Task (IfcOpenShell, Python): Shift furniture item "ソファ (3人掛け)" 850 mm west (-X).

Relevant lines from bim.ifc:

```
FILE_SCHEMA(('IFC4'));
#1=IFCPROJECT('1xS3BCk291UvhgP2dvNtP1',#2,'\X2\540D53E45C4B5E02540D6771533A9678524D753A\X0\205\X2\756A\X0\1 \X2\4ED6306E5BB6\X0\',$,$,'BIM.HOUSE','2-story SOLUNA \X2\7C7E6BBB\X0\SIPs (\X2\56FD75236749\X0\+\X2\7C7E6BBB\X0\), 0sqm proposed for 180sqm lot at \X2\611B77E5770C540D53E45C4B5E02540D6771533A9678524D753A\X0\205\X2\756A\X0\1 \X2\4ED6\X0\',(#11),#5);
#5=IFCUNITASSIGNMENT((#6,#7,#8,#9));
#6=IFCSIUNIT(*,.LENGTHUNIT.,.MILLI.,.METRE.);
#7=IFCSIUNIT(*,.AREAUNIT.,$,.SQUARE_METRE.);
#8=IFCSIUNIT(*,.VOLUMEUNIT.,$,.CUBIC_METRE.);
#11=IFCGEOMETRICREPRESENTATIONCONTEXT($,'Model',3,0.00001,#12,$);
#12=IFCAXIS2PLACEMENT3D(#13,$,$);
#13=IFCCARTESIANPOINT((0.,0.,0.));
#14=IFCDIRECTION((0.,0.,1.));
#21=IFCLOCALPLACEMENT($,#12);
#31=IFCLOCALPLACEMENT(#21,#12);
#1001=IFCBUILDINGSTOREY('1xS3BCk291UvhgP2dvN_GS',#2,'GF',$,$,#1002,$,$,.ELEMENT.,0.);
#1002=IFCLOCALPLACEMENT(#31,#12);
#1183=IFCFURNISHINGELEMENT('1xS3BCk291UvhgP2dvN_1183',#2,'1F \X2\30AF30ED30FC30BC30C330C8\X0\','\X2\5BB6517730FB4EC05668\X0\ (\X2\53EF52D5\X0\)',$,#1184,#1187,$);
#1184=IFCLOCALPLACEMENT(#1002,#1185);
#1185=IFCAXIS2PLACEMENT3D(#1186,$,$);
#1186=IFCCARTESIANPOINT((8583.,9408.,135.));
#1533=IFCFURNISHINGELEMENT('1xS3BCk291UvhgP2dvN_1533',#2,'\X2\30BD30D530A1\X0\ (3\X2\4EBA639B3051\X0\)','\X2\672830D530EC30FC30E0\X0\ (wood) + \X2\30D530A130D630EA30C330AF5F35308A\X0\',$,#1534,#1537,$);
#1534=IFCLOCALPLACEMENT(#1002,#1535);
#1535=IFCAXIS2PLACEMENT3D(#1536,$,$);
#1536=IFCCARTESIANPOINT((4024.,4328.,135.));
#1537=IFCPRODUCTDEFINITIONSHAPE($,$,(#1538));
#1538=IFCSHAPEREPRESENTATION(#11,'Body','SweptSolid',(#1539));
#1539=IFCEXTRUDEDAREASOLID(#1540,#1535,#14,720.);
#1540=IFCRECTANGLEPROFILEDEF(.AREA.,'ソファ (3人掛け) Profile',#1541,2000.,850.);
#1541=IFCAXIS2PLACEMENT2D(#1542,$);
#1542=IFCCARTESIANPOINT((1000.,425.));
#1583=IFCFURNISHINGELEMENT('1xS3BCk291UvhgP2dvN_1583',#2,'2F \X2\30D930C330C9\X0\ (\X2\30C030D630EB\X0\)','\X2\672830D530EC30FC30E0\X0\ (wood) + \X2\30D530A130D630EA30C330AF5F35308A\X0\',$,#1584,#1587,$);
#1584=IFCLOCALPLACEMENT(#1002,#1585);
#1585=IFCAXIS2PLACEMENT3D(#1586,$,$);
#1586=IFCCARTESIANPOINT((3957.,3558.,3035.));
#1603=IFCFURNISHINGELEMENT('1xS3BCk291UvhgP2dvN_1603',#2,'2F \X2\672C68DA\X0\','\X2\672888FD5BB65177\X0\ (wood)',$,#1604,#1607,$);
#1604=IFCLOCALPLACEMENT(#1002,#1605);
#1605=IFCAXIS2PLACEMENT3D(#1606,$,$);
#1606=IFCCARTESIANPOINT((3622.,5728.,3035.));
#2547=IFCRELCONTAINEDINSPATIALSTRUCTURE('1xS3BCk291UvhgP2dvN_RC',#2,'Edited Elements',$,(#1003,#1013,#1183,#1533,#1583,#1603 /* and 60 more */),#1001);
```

```python
import ifcopenshell
import ifcopenshell.api.geometry
import ifcopenshell.util.placement

model = ifcopenshell.open("bim.ifc")

item = model.by_guid("1xS3BCk291UvhgP2dvN_1533")
matrix = ifcopenshell.util.placement.get_local_placement(item.ObjectPlacement)
matrix[0, 3] -= 850.0
ifcopenshell.api.geometry.edit_object_placement(model, product=item, matrix=matrix, is_si=False)

print(ifcopenshell.util.placement.get_local_placement(item.ObjectPlacement).round(3) + 0.0)

model.write("bim_rev.ifc")
```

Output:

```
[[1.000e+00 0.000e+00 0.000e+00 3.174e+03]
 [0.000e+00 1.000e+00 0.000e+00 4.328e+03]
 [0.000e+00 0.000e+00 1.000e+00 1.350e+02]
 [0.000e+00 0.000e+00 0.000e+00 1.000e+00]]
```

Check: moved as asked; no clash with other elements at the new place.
